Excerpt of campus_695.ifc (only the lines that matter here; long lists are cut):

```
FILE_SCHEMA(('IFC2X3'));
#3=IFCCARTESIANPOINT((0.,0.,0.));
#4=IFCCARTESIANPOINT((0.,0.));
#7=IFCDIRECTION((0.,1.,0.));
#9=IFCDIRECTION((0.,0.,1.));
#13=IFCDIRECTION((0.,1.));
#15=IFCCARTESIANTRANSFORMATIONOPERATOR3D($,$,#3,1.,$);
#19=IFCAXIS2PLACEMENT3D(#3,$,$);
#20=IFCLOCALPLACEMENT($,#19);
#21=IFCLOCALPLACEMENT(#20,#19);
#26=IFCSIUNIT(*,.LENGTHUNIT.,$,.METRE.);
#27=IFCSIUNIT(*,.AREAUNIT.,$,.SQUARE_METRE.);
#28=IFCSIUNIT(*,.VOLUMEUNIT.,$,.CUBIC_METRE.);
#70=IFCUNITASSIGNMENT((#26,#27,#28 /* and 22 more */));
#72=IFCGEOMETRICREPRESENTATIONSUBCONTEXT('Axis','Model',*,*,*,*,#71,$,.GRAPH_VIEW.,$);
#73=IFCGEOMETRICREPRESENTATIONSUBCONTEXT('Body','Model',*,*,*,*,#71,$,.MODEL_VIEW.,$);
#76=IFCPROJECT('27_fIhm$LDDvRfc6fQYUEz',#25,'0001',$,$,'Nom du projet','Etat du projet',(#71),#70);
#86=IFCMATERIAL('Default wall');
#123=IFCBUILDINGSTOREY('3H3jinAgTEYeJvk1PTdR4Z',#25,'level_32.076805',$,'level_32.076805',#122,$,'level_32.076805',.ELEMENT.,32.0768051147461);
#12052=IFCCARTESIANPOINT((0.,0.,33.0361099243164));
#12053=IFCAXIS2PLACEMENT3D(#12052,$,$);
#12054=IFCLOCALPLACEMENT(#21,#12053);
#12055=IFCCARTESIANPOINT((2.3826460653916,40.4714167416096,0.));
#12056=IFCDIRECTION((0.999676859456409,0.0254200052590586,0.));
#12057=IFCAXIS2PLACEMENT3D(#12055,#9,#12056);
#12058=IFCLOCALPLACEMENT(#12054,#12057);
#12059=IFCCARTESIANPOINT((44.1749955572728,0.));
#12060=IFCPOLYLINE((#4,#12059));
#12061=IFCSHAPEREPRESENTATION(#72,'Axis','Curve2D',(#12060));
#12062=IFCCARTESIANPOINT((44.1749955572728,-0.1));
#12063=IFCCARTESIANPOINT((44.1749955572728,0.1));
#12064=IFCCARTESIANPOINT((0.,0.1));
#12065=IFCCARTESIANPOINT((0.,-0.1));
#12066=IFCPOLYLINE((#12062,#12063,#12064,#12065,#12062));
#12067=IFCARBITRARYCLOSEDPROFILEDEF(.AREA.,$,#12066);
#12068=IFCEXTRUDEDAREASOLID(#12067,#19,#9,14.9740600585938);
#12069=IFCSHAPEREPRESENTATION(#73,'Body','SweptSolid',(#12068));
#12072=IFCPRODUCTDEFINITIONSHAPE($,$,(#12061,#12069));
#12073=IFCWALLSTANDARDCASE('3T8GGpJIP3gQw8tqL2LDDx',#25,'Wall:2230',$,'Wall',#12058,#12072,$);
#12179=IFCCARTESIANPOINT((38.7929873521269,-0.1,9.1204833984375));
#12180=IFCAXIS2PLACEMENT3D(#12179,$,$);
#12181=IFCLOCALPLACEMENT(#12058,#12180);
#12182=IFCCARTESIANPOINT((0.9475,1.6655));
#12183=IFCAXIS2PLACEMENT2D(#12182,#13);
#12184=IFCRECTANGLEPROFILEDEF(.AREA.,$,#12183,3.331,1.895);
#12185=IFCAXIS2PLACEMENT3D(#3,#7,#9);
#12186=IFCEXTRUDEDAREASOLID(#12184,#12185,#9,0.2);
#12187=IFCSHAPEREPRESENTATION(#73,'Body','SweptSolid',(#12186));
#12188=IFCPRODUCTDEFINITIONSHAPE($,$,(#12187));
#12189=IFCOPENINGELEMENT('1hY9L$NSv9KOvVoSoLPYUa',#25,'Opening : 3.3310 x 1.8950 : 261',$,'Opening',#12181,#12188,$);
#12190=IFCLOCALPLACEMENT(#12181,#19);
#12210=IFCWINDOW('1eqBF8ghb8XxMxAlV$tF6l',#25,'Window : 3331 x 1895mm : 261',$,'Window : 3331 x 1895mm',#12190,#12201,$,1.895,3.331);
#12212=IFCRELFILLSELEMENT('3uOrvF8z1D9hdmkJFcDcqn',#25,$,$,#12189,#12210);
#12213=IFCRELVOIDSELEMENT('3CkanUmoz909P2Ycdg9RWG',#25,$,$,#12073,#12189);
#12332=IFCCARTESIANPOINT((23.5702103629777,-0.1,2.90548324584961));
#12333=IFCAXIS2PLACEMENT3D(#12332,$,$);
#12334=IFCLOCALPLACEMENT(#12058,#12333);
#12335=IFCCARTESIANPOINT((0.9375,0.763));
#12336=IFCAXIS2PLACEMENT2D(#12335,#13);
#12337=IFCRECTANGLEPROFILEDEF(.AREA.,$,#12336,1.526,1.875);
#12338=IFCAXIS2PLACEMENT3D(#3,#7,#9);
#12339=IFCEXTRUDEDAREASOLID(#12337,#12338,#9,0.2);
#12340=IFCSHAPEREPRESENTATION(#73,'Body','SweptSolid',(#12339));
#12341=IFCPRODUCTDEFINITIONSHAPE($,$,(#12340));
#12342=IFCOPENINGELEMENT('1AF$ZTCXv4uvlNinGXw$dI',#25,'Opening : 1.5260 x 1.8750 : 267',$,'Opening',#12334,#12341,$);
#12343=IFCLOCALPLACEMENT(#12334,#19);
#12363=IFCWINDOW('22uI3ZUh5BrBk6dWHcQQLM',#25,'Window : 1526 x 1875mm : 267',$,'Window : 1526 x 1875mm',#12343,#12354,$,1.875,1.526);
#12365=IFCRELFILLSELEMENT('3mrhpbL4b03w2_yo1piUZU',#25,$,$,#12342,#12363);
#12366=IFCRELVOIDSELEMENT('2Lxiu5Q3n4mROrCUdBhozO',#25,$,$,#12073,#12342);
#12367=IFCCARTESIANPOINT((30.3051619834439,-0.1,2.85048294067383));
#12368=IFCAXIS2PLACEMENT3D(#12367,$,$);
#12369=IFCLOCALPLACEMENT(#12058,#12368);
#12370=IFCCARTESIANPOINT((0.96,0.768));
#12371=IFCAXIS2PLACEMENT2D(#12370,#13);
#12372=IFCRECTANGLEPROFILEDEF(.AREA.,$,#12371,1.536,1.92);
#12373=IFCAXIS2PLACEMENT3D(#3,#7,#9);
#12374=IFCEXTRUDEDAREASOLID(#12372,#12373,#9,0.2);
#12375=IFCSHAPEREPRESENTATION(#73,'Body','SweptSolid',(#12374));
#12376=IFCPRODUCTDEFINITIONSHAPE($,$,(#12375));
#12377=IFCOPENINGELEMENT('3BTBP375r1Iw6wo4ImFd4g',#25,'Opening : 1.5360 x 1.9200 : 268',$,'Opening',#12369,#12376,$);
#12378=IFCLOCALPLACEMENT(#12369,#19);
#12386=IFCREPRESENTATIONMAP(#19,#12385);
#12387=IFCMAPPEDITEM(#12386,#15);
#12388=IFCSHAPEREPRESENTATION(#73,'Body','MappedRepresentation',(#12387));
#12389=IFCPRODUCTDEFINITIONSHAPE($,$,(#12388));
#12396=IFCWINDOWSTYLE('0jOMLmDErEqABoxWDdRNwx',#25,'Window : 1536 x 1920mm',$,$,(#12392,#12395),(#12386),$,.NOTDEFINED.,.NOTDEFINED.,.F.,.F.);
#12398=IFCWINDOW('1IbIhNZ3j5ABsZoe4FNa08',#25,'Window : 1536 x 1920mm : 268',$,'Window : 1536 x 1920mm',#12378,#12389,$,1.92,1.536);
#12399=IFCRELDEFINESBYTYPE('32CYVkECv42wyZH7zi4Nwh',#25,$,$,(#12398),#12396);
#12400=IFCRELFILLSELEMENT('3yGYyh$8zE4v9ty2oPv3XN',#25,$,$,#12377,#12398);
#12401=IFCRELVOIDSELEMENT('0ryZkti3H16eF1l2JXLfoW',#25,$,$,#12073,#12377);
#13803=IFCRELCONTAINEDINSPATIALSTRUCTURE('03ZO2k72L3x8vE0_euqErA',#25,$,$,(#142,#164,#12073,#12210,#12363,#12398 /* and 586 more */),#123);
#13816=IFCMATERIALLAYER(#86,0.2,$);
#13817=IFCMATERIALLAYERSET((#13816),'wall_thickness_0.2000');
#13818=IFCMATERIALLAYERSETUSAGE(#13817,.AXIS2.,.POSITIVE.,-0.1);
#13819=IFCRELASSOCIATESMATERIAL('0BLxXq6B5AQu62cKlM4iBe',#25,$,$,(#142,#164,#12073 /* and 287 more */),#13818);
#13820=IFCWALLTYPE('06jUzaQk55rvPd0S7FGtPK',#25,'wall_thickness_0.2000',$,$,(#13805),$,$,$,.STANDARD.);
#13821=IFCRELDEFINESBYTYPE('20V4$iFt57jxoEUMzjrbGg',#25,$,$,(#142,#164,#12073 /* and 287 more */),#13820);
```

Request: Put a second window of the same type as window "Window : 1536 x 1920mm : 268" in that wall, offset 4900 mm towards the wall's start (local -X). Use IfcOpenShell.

```python
import ifcopenshell
import ifcopenshell.api.feature
import ifcopenshell.api.geometry
import ifcopenshell.api.root
import ifcopenshell.geom
import ifcopenshell.util.element
import ifcopenshell.util.placement
import ifcopenshell.util.shape

model = ifcopenshell.open("campus_695.ifc")
settings = ifcopenshell.geom.settings()


def volume(element):
    """Net volume in cubic metres, openings subtracted."""
    shape = ifcopenshell.geom.create_shape(settings, element)
    return ifcopenshell.util.shape.get_volume(shape.geometry)


window = model.by_id(12398)
opening = window.FillsVoids[0].RelatingOpeningElement
wall = opening.VoidsElements[0].RelatingBuildingElement
before = volume(wall)
shift = ifcopenshell.util.placement.get_local_placement(wall.ObjectPlacement)[:3, 0] * -4.9

# copy_class copies the void relationship, type, container and properties, but no geometry.
new_opening = ifcopenshell.api.root.copy_class(model, product=opening)
new_opening.Representation = ifcopenshell.util.element.copy_deep(
    model, opening.Representation, exclude=["IfcGeometricRepresentationContext", "IfcRepresentationMap"]
)
new_opening.Name = "Opening : 1.5360 x 1.9200"
new_window = ifcopenshell.api.root.copy_class(model, product=window)
new_window.Representation = ifcopenshell.util.element.copy_deep(
    model, window.Representation, exclude=["IfcGeometricRepresentationContext", "IfcRepresentationMap"]
)
new_window.Name = "Window : 1536 x 1920mm"
fills = ifcopenshell.api.feature.add_filling(model, opening=new_opening, element=new_window)
fills.OwnerHistory = new_window.OwnerHistory  # required in IFC2X3

for old, new in ((opening, new_opening), (window, new_window)):
    matrix = ifcopenshell.util.placement.get_local_placement(old.ObjectPlacement)
    matrix[:3, 3] += shift
    ifcopenshell.api.geometry.edit_object_placement(model, product=new, matrix=matrix, is_si=False)

after = volume(wall)

print(f"wall volume {before:.3f} -> {after:.3f} m3")

model.write("campus_695_v2.ifc")
```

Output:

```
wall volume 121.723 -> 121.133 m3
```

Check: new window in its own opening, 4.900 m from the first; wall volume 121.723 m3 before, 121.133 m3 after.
